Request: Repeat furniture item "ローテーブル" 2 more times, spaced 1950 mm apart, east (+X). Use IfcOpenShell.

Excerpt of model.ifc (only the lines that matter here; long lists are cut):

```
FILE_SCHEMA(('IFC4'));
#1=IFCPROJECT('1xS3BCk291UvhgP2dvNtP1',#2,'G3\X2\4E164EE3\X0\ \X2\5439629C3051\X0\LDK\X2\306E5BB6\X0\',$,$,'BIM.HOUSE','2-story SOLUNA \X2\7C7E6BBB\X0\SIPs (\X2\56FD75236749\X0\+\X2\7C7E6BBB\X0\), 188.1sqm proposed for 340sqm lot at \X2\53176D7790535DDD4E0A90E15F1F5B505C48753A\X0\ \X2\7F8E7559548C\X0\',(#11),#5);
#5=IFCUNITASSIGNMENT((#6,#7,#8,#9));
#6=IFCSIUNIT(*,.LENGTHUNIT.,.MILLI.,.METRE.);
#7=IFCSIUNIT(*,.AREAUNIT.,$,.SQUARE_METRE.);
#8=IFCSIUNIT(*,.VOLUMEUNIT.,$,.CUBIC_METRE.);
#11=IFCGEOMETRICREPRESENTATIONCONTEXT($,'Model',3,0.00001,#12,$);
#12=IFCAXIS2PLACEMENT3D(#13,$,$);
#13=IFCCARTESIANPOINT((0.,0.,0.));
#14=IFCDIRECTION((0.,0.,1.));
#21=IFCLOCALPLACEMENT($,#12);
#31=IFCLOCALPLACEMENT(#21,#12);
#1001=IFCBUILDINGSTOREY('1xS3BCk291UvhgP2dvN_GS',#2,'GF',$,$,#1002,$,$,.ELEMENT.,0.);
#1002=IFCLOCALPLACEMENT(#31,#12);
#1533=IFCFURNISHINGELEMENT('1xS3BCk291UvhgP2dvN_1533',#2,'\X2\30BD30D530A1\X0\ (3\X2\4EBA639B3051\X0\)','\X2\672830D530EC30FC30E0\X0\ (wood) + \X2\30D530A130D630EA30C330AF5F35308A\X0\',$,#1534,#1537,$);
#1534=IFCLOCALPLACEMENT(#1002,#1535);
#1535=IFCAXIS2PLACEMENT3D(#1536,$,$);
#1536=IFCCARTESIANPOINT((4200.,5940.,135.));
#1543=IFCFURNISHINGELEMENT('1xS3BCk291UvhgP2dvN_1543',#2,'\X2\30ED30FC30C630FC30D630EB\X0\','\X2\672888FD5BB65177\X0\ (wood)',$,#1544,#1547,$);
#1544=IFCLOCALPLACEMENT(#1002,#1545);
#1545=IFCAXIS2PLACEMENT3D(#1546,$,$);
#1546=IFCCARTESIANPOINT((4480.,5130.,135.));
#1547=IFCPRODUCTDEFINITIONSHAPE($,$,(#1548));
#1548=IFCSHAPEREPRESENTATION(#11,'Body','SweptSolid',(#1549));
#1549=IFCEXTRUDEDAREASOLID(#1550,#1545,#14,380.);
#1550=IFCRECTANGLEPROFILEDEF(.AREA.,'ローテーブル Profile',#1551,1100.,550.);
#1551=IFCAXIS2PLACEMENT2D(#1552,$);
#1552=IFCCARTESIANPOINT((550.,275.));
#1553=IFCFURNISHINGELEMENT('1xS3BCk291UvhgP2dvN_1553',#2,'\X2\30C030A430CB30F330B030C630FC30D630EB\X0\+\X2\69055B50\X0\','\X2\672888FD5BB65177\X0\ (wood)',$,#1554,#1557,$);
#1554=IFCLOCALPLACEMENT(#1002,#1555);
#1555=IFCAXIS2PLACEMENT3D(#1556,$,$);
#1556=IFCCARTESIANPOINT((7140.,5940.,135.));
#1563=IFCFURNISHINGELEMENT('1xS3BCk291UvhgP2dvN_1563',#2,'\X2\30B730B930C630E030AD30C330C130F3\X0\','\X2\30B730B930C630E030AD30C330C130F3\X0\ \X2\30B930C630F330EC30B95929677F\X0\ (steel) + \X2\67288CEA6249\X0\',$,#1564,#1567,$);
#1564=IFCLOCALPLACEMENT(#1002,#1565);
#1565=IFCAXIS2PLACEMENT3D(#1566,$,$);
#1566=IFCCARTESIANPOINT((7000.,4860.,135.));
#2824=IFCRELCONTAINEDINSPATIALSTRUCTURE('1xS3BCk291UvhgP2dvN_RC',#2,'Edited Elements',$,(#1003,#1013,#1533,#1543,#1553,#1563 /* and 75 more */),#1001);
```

```python
import numpy as np
import ifcopenshell
import ifcopenshell.api.geometry
import ifcopenshell.api.root
import ifcopenshell.util.element
import ifcopenshell.util.placement
import ifcopenshell.util.unit

model = ifcopenshell.open("model.ifc")
unit_scale = ifcopenshell.util.unit.calculate_unit_scale(model)


def reuse_history(source, copy):
    """copy_class also copies each property set's owner history, people and application; keep the originals."""
    for rel in copy.IsDefinedBy:
        if rel.is_a("IfcRelDefinesByProperties") and (history := rel.RelatingPropertyDefinition.OwnerHistory):
            rel.RelatingPropertyDefinition.OwnerHistory = source.OwnerHistory
            ifcopenshell.util.element.remove_deep2(model, history)


source = model.by_guid("1xS3BCk291UvhgP2dvN_1543")
base = ifcopenshell.util.placement.get_local_placement(source.ObjectPlacement)
step = np.array([1.0, 0.0, 0.0]) * 1.95 / unit_scale

for i in range(1, 3):
    copy = ifcopenshell.api.root.copy_class(model, product=source)
    copy.Representation = ifcopenshell.util.element.copy_deep(
        model, source.Representation, exclude=["IfcGeometricRepresentationContext", "IfcRepresentationMap"]
    )
    reuse_history(source, copy)
    matrix = base.copy()
    matrix[:3, 3] += i * step
    print("added at", matrix[:3, 3].round(3) + 0.0)
    ifcopenshell.api.geometry.edit_object_placement(model, product=copy, matrix=matrix, is_si=False)

model.write("model_updated.ifc")
```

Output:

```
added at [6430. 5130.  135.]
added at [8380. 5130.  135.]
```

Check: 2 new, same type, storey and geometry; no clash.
